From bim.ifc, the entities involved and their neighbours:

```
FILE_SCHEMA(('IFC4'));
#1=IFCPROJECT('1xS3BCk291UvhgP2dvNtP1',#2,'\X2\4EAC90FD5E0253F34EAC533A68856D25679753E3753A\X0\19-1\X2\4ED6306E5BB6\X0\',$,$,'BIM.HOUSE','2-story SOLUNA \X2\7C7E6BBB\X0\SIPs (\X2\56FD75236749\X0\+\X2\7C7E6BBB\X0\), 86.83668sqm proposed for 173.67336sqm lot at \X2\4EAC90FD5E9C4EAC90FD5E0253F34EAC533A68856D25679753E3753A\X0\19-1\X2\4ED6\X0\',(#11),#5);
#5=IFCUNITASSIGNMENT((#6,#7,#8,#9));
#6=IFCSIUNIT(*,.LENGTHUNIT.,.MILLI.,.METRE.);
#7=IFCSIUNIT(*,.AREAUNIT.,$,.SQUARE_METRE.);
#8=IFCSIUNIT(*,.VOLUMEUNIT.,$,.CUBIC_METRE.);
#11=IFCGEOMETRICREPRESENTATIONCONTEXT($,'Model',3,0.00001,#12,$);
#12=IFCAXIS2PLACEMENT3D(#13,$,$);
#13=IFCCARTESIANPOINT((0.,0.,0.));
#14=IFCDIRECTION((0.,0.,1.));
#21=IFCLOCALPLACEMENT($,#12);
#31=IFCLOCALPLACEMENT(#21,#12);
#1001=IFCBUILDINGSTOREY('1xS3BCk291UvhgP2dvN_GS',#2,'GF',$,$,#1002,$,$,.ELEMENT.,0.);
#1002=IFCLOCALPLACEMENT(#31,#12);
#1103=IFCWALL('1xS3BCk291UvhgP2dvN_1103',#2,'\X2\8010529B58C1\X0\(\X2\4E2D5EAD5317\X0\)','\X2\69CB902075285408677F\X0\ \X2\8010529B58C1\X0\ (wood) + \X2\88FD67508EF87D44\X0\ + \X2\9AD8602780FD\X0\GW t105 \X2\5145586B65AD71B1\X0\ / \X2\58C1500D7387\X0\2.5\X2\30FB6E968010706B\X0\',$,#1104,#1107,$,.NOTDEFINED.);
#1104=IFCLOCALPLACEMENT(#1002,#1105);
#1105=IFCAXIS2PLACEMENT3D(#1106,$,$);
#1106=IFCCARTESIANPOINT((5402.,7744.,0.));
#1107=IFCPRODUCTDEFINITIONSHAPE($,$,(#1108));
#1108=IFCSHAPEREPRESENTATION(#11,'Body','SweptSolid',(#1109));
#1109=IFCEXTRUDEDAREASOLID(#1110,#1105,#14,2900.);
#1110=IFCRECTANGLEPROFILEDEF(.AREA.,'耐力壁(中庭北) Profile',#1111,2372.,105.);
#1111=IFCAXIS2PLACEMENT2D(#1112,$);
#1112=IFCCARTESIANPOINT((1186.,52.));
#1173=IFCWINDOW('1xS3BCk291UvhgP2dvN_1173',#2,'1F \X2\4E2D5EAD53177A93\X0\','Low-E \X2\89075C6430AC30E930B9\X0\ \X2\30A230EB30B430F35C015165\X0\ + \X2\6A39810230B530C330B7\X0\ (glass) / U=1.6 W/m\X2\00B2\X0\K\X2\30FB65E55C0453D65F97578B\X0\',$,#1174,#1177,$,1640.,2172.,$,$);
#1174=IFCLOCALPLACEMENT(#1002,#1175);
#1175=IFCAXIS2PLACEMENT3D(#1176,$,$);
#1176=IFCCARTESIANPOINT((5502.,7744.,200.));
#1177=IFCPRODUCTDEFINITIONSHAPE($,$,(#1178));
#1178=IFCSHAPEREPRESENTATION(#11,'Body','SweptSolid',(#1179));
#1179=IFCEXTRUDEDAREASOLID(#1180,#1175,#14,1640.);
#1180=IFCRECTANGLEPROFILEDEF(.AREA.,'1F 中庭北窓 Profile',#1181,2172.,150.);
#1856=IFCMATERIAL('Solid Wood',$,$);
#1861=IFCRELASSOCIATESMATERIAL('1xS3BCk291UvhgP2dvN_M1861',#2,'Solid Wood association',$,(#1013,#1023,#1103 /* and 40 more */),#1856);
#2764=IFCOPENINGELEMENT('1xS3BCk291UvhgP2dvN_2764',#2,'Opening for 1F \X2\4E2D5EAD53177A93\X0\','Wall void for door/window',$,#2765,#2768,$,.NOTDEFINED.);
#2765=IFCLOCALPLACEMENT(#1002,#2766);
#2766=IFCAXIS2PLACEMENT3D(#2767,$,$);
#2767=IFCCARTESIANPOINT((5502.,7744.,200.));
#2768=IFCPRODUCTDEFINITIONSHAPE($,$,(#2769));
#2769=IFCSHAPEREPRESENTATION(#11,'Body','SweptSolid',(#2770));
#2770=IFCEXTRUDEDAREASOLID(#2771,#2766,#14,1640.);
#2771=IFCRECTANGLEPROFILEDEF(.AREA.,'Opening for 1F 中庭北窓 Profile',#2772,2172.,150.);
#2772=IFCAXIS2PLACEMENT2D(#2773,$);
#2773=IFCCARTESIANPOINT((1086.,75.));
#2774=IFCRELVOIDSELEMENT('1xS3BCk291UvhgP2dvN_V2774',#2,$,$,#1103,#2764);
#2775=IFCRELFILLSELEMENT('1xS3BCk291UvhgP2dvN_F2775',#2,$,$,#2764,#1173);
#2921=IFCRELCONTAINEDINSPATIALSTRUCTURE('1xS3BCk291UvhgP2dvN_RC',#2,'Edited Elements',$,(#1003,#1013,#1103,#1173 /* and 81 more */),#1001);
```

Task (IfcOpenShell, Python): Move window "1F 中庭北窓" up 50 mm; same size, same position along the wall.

```python
import numpy as np
import ifcopenshell
import ifcopenshell.api.geometry
import ifcopenshell.util.placement
import ifcopenshell.util.unit

model = ifcopenshell.open("bim.ifc")
unit_scale = ifcopenshell.util.unit.calculate_unit_scale(model)

window = model.by_guid("1xS3BCk291UvhgP2dvN_1173")
opening = window.FillsVoids[0].RelatingOpeningElement
dz = 0.05 / unit_scale

shift = np.array([0.0, 0.0, dz])
# The window is not placed relative to its opening, so move both.
for product in (opening, window):
    matrix = ifcopenshell.util.placement.get_local_placement(product.ObjectPlacement)
    matrix[:3, 3] += shift
    ifcopenshell.api.geometry.edit_object_placement(model, product=product, matrix=matrix, is_si=False)

print(f"moved by {dz * unit_scale:+.3f} m")

model.write("bim_rev.ifc")
```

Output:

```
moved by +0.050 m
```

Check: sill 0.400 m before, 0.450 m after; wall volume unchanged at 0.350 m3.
